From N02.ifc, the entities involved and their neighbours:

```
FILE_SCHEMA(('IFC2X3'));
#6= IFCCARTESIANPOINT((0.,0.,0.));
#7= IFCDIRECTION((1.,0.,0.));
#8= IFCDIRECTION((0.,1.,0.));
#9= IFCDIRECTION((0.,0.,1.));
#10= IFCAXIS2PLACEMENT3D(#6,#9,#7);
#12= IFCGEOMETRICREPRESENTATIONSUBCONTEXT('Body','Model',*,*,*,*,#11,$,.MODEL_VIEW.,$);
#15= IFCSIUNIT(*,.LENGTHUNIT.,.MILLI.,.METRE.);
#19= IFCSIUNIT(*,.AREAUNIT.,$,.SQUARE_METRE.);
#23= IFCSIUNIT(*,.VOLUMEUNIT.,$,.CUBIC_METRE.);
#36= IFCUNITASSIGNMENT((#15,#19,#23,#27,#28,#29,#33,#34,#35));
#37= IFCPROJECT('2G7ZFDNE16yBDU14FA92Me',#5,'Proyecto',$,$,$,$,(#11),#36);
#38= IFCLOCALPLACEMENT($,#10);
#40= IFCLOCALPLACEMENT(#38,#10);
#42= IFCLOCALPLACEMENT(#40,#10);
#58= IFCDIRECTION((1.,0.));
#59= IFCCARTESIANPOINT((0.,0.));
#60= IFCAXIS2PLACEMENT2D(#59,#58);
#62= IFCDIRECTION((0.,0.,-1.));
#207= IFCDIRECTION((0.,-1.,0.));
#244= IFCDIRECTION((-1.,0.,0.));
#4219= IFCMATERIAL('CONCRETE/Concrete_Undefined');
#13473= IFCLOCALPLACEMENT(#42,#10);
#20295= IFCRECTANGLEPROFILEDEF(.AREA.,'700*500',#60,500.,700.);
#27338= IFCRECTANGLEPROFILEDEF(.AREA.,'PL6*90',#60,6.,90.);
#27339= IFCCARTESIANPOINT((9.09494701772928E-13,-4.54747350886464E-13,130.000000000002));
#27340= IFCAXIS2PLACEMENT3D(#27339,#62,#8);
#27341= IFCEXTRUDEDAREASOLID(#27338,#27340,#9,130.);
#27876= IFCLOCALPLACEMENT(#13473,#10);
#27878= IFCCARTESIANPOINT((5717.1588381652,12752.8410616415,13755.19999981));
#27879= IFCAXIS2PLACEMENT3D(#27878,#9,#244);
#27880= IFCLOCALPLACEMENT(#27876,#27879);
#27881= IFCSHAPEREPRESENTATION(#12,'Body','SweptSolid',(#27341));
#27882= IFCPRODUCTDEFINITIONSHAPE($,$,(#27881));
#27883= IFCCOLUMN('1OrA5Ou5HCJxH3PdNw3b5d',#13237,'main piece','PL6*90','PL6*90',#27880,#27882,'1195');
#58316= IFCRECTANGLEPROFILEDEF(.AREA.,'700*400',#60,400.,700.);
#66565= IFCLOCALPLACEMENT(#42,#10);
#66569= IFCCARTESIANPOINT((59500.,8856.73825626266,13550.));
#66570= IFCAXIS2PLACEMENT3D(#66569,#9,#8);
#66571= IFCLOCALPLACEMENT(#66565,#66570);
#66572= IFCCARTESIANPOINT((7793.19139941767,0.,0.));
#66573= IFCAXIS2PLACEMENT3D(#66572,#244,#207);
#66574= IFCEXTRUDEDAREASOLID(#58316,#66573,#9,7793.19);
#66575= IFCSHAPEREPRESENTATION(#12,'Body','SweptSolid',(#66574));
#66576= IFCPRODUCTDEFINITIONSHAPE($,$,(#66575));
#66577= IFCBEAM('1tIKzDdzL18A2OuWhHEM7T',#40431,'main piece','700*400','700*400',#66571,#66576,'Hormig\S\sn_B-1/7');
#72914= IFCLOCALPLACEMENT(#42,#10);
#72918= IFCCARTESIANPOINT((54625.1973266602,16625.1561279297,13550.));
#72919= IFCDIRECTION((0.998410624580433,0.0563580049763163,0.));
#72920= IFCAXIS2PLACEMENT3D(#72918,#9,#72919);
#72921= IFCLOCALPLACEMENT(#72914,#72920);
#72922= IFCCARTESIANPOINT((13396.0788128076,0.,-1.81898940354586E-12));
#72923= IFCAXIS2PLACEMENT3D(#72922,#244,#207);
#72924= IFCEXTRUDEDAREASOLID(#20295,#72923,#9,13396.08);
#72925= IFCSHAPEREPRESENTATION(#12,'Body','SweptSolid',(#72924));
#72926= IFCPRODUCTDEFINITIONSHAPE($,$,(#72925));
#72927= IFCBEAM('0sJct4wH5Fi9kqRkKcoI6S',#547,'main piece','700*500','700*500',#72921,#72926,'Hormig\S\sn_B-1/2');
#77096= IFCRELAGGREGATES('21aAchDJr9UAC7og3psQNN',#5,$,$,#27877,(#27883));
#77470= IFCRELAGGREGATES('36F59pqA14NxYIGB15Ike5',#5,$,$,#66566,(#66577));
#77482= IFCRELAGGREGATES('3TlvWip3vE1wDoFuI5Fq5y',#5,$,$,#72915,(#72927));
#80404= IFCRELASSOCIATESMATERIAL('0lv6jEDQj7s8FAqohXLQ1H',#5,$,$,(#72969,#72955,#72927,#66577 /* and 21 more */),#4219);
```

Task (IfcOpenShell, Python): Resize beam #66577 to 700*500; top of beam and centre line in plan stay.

```python
import ifcopenshell
import ifcopenshell.util.element
import ifcopenshell.util.representation

model = ifcopenshell.open("N02.ifc")

member = model.by_guid("1tIKzDdzL18A2OuWhHEM7T")
source = next(p for p in model.by_type("IfcRectangleProfileDef") if p.ProfileName == "700*500")

body = ifcopenshell.util.representation.get_representation(member, "Model", "Body")
solid = body.Items[0]
old_profile = solid.SweptArea

# Copy the section's sizes but keep this member's own profile position.
profile = ifcopenshell.util.element.copy(model, source)
# Profiles are centred, so shift by half the change in depth to hold the top.
shift = (old_profile.YDim - profile.YDim) / 2
x, y = old_profile.Position.Location.Coordinates
up = (0.0, 1.0)  # upwards, in the solid's own plane
location = model.createIfcCartesianPoint((x + up[0] * shift, y + up[1] * shift))
profile.Position = model.createIfcAxis2Placement2D(location, old_profile.Position.RefDirection)
solid.SweptArea = profile
if not model.get_total_inverses(old_profile):
    ifcopenshell.util.element.remove_deep2(model, old_profile)
member.Description = member.Description.replace("700*400", "700*500")
member.ObjectType = member.ObjectType.replace("700*400", "700*500")

print(solid.SweptArea)

model.write("N02_rev.ifc")
```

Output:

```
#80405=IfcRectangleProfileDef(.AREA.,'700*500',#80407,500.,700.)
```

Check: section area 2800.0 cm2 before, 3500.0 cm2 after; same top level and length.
